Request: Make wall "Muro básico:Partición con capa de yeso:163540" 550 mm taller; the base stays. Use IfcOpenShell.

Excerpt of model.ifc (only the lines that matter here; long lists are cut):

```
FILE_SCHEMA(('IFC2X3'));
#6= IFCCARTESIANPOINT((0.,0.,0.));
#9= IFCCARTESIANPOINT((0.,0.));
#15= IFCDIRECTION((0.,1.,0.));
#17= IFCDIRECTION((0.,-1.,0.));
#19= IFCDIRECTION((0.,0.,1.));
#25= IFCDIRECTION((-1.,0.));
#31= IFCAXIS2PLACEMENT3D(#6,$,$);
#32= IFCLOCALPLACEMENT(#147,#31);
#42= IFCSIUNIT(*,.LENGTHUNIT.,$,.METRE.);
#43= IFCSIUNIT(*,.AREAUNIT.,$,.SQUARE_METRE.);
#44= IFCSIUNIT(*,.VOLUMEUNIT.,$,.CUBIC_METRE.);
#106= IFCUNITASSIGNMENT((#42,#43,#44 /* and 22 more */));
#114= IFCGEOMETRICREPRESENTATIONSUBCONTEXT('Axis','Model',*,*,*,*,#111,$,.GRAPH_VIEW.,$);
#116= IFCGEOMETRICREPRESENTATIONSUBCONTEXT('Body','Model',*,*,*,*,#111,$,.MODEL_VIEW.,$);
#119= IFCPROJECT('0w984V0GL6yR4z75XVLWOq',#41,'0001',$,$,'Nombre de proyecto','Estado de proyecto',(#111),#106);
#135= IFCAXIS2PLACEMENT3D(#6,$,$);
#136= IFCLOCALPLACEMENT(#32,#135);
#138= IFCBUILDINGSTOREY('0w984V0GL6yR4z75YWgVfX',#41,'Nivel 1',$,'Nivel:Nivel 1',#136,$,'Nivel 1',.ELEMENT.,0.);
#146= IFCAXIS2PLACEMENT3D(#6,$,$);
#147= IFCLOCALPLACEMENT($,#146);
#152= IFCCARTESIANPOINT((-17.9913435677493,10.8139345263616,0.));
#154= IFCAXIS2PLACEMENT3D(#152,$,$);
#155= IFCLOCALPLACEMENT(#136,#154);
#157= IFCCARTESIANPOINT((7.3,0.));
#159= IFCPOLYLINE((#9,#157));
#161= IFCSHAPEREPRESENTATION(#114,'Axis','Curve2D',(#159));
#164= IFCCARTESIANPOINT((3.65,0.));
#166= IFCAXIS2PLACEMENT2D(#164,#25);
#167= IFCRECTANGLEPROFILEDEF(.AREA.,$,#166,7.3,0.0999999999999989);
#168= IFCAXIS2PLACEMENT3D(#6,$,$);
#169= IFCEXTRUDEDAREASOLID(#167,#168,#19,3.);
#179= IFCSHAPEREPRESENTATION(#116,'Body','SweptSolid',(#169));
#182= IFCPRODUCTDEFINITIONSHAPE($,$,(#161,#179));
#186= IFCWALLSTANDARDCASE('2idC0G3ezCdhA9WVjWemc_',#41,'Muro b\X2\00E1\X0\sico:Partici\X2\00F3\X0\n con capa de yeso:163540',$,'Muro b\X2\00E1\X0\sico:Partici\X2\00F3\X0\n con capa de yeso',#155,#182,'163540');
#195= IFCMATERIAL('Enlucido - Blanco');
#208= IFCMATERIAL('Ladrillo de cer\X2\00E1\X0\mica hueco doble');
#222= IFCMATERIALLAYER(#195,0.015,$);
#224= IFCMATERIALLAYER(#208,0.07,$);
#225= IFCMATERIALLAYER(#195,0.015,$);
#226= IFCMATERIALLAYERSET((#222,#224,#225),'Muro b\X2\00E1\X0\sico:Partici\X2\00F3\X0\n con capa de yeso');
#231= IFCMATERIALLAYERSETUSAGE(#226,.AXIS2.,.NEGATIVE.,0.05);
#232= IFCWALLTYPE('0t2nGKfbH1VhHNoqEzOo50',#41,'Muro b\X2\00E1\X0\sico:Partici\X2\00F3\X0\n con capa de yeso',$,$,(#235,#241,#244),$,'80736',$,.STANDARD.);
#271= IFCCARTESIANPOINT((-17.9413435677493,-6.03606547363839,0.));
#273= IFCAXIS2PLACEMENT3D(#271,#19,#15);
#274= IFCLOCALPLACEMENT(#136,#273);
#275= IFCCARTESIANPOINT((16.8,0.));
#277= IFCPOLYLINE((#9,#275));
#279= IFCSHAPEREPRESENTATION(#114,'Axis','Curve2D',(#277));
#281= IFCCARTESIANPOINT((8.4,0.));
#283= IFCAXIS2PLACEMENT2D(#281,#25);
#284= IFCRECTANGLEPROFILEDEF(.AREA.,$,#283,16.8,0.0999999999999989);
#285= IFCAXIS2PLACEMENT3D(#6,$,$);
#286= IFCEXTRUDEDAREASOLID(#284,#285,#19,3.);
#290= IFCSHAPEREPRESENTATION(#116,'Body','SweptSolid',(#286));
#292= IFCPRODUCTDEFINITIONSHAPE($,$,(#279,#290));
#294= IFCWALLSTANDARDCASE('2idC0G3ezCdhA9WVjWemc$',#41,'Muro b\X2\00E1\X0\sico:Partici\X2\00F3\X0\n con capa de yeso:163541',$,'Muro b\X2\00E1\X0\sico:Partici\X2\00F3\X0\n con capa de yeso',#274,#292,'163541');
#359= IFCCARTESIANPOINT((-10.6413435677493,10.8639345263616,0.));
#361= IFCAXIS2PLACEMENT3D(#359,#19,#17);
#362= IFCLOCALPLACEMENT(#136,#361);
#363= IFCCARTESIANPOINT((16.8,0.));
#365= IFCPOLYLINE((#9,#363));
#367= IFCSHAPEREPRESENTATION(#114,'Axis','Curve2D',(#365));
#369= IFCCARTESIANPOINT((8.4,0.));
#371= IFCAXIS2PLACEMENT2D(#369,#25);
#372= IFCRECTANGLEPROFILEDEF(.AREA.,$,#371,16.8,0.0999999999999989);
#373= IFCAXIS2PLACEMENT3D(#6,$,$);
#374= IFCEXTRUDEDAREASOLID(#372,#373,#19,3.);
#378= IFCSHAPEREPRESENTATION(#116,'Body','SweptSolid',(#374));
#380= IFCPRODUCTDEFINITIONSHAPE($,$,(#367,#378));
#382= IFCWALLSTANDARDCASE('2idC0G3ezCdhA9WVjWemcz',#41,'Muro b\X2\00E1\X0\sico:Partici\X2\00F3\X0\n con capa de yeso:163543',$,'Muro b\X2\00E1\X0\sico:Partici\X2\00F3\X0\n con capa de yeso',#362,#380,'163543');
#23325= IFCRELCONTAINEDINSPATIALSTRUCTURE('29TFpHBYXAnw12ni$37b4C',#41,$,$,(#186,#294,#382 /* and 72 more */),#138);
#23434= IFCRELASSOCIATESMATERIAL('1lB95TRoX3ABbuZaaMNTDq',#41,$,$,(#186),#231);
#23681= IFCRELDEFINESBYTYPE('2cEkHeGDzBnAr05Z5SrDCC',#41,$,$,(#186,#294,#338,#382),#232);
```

```python
import ifcopenshell
import ifcopenshell.geom
import ifcopenshell.util.representation
import ifcopenshell.util.shape

model = ifcopenshell.open("model.ifc")
settings = ifcopenshell.geom.settings()


def volume(element):
    """Net volume in cubic metres, openings subtracted."""
    shape = ifcopenshell.geom.create_shape(settings, element)
    return ifcopenshell.util.shape.get_volume(shape.geometry)


wall = model.by_guid("2idC0G3ezCdhA9WVjWemc_")
before = volume(wall)

body = ifcopenshell.util.representation.get_representation(wall, "Model", "Body")
solid = body.Items[0]
old_height = solid.Depth
solid.Depth += 0.55
after = volume(wall)

print(f"height {old_height:g} -> {solid.Depth:g}, volume {before:.3f} -> {after:.3f} m3")

model.write("model_edited.ifc")
```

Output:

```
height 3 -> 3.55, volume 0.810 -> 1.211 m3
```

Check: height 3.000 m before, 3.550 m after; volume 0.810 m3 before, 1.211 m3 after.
